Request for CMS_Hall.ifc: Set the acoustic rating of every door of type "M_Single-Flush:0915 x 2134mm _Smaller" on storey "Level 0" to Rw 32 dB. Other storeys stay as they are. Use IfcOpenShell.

First a look at what the model holds.

```python
import ifcopenshell
import ifcopenshell.util.element

model = ifcopenshell.open("CMS_Hall.ifc")
print(model.schema)
storey = next(s for s in model.by_type("IfcBuildingStorey") if s.Name == "Level 0")
doors = [e for e in ifcopenshell.util.element.get_decomposition(storey) if e.is_a("IfcDoor")]
seen = {}
for e in doors:
    element_type = ifcopenshell.util.element.get_type(e)
    key = (element_type.Name if element_type != e and element_type else None, ifcopenshell.util.element.get_pset(e, "Pset_DoorCommon", "AcousticRating"))
    seen[key] = seen.get(key, 0) + 1
for (name, value), count in sorted(seen.items(), key=str):
    print(count, "x", name, "|", value)
```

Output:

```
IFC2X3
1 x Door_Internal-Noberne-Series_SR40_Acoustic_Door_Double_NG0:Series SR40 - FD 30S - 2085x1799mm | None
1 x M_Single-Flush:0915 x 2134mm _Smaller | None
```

```python
import ifcopenshell
import ifcopenshell.api.pset
import ifcopenshell.util.element

model = ifcopenshell.open("CMS_Hall.ifc")

storey = next(s for s in model.by_type("IfcBuildingStorey") if s.Name == "Level 0")
doors = [e for e in ifcopenshell.util.element.get_decomposition(storey) if e.is_a("IfcDoor")]

count = 0
for e in doors:
    element_type = ifcopenshell.util.element.get_type(e)
    if element_type in (None, e) or element_type.Name != "M_Single-Flush:0915 x 2134mm _Smaller":
        continue
    # add_pset returns the element's existing set when there is one.
    pset = ifcopenshell.api.pset.add_pset(model, product=e, name="Pset_DoorCommon")
    ifcopenshell.api.pset.edit_pset(model, pset=pset, properties={"AcousticRating": "Rw 32 dB"})
    count += 1

print(count, "doors updated")

model.write("CMS_Hall_v2.ifc")
```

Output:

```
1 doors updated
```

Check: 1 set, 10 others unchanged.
